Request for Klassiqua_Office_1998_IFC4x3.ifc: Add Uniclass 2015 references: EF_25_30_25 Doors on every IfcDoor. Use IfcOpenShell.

First a look at what the model holds.

```python
import ifcopenshell

model = ifcopenshell.open("Klassiqua_Office_1998_IFC4x3.ifc")
print(model.schema)
print("classifications:", [c.Name for c in model.by_type("IfcClassification")])
for ifc_class in ("IfcDoor", "IfcRoof", "IfcStair", "IfcWall", "IfcWindow"):
    print(ifc_class, len(model.by_type(ifc_class)))
```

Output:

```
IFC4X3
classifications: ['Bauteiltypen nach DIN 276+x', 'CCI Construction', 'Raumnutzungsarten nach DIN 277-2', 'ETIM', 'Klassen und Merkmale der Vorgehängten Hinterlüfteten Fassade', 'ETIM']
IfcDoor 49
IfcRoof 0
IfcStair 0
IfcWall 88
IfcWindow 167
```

```python
import ifcopenshell
import ifcopenshell.api.classification

model = ifcopenshell.open("Klassiqua_Office_1998_IFC4x3.ifc")

system = ifcopenshell.api.classification.add_classification(model, classification="Uniclass 2015")

codes = {
    "IfcDoor": ("EF_25_30_25", "Doors"),
}
for ifc_class, (code, name) in codes.items():
    products = model.by_type(ifc_class)
    ifcopenshell.api.classification.add_reference(
        model, products=products, classification=system, identification=code, name=name
    )
    print(code, len(products))

model.write("Klassiqua_Office_1998_IFC4x3_updated.ifc")
```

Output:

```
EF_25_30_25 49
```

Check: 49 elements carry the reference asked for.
